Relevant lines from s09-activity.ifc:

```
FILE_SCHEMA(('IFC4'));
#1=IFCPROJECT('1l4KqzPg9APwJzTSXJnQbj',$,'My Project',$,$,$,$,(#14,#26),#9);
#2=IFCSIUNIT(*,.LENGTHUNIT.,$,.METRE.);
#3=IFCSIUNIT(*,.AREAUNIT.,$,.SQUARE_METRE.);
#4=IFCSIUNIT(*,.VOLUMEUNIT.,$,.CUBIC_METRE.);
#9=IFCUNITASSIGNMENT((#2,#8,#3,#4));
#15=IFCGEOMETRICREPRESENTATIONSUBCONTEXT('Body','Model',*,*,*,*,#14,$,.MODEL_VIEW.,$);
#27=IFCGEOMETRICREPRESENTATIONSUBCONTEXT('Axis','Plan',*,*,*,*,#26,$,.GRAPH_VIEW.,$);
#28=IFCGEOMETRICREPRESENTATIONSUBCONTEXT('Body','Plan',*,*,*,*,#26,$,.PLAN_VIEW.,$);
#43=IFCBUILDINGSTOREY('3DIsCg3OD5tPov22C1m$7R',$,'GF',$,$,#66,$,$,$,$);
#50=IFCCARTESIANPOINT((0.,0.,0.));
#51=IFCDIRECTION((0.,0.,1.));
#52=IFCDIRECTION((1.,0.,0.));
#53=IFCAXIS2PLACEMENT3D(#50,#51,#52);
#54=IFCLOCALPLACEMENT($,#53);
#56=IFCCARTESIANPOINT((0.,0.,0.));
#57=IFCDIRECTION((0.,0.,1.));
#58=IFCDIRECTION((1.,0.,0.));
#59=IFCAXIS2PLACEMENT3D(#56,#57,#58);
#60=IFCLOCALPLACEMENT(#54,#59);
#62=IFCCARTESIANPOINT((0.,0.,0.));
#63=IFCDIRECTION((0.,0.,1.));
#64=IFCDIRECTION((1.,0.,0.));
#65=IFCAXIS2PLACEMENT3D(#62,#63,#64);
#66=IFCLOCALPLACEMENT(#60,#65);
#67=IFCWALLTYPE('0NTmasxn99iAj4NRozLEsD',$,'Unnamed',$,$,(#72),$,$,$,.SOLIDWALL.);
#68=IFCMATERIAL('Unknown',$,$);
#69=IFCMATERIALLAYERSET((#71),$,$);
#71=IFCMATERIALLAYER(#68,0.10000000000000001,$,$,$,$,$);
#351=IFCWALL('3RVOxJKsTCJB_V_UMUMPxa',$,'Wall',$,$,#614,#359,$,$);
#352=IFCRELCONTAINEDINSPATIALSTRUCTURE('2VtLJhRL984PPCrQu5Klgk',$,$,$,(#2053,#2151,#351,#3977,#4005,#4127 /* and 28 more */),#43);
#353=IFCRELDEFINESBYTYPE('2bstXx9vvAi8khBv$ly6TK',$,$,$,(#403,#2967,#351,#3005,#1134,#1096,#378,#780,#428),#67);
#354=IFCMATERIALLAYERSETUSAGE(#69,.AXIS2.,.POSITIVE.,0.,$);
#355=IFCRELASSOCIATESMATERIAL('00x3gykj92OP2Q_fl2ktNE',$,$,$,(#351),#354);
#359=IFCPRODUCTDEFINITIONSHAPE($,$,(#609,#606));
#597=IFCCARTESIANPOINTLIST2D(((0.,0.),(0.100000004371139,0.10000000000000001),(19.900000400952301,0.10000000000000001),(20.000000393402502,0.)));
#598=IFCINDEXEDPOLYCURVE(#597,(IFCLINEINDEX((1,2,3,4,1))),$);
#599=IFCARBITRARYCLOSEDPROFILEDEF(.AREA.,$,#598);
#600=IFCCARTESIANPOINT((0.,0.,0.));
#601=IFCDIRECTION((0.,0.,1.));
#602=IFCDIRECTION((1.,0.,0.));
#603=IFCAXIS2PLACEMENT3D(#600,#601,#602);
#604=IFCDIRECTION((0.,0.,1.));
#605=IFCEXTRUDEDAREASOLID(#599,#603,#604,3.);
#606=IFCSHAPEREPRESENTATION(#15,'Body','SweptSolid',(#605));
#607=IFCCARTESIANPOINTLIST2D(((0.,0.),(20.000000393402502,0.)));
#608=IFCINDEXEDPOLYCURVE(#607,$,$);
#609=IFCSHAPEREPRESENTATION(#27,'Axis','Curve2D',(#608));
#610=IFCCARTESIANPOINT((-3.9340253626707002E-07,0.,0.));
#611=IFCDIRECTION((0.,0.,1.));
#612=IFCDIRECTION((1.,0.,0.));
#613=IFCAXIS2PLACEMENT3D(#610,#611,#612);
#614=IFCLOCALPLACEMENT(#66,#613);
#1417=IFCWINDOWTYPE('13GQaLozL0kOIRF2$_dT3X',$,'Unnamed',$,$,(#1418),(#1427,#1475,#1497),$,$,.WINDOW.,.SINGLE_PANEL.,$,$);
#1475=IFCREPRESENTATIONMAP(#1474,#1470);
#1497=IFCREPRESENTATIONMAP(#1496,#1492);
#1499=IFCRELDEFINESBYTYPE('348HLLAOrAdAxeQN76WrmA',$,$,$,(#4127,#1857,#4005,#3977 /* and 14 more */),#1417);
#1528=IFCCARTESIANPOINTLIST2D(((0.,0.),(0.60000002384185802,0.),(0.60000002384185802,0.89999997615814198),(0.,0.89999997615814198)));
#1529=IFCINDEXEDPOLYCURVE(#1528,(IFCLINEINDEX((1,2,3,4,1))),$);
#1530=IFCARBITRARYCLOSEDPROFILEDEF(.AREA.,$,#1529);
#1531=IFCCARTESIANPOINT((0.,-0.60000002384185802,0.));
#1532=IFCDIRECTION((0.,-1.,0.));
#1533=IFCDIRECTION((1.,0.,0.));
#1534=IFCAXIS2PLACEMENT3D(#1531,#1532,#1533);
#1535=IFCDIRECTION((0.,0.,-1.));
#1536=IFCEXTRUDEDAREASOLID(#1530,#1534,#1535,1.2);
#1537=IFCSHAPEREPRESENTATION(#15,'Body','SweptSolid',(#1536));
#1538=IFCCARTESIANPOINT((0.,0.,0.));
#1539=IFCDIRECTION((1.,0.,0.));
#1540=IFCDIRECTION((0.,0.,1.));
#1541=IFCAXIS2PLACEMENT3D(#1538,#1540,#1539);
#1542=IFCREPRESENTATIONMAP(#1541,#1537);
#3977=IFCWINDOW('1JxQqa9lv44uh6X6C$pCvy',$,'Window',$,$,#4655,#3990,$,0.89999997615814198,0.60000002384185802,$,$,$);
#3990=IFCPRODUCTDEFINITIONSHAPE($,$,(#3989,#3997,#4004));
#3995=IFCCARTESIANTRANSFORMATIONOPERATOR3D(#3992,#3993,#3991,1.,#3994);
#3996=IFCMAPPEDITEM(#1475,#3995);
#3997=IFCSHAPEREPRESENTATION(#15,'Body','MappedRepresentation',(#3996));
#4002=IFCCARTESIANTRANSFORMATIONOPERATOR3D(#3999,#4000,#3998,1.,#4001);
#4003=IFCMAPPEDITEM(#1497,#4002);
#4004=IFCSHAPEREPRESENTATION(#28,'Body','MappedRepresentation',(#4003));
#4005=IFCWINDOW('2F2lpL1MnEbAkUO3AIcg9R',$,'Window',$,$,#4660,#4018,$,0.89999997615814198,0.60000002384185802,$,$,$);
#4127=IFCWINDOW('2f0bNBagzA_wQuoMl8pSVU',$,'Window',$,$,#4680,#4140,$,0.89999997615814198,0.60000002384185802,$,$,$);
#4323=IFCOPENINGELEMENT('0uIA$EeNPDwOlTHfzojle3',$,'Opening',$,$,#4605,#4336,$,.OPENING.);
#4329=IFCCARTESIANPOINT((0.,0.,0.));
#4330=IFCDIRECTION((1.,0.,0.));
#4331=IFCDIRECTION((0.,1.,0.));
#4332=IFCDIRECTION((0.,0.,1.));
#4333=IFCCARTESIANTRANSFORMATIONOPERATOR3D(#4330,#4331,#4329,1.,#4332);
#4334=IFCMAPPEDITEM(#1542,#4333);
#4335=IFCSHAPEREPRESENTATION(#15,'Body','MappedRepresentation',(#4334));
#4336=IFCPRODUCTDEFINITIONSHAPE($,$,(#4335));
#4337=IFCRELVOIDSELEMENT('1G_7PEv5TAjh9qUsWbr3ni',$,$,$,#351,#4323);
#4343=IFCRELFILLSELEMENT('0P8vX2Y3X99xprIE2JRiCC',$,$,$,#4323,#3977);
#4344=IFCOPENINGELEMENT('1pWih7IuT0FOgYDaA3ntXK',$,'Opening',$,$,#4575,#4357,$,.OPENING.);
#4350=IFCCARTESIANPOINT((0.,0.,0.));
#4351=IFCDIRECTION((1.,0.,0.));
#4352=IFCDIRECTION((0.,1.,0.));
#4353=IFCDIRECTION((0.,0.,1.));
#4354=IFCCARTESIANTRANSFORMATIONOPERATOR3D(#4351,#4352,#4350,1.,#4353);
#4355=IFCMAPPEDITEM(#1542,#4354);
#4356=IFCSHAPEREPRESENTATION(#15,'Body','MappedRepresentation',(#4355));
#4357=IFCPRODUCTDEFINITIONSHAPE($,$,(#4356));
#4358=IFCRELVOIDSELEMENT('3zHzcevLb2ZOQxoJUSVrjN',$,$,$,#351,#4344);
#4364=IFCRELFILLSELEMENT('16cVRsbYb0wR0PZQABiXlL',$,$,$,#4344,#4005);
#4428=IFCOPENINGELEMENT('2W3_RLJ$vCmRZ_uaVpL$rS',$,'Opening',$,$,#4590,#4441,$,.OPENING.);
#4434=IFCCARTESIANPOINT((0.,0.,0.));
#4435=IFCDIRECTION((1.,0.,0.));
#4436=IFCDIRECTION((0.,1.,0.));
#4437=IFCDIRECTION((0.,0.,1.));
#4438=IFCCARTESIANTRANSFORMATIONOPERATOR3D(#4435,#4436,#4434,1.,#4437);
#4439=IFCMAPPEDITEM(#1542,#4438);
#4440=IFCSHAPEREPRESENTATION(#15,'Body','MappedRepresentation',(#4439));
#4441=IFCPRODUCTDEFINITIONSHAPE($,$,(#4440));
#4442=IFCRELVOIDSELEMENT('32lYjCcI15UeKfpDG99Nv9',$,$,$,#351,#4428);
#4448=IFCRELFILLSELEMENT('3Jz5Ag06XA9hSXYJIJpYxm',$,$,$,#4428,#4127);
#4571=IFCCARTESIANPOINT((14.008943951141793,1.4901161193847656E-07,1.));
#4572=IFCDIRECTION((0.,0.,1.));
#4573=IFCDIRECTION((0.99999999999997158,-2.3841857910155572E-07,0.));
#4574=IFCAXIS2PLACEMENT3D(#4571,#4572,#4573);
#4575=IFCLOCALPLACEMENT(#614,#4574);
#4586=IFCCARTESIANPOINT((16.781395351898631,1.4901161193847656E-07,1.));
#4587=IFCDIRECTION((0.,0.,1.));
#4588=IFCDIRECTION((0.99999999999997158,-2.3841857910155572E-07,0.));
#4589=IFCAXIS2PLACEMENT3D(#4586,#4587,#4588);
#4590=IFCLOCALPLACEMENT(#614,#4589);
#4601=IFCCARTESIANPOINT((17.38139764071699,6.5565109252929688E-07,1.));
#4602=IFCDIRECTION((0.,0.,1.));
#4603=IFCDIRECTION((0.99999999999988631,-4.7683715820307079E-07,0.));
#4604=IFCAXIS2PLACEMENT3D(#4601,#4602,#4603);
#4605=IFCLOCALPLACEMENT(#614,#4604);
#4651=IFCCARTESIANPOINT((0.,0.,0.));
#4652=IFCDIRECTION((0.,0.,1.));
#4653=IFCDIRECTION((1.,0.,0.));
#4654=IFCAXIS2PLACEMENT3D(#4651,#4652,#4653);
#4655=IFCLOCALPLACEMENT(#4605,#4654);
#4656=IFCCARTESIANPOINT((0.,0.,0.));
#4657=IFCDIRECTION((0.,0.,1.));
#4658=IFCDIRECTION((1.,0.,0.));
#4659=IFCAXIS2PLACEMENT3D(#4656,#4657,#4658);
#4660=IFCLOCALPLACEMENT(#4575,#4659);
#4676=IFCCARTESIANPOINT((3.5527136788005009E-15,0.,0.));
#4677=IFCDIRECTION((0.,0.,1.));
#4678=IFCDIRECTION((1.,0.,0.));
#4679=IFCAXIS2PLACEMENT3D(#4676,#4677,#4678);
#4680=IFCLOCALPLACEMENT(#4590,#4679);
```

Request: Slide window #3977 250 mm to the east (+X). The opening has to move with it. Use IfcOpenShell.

```python
import ifcopenshell
import ifcopenshell.api.geometry
import ifcopenshell.util.placement
import ifcopenshell.util.unit

model = ifcopenshell.open("s09-activity.ifc")
unit_scale = ifcopenshell.util.unit.calculate_unit_scale(model)

window = model.by_id(3977)
opening = window.FillsVoids[0].RelatingOpeningElement
wall = opening.VoidsElements[0].RelatingBuildingElement

wall_matrix = ifcopenshell.util.placement.get_local_placement(wall.ObjectPlacement)
shift = wall_matrix[:3, 0] * 0.25 / unit_scale
before = ifcopenshell.util.placement.get_local_placement(window.ObjectPlacement)[:3, 3].copy()

# The window is placed relative to its opening, so it follows when the opening moves.
matrix = ifcopenshell.util.placement.get_local_placement(opening.ObjectPlacement)
matrix[:3, 3] += shift
ifcopenshell.api.geometry.edit_object_placement(
    model, product=opening, matrix=matrix, is_si=False, should_transform_children=True
)

after = ifcopenshell.util.placement.get_local_placement(window.ObjectPlacement)[:3, 3]
print("window moved by", (after - before).round(3) + 0.0)

model.write("s09-activity_edited.ifc")
```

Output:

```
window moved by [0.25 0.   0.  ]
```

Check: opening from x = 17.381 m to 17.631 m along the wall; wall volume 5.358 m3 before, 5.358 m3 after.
